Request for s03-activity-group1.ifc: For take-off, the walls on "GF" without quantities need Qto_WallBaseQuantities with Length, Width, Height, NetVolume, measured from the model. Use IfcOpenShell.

First a look at what the model holds.

```python
import ifcopenshell
import ifcopenshell.util.element
import ifcopenshell.util.unit

model = ifcopenshell.open("s03-activity-group1.ifc")
print(model.schema)
for unit_type in ("LENGTHUNIT", "AREAUNIT", "VOLUMEUNIT"):
    print(unit_type, ifcopenshell.util.unit.calculate_unit_scale(model, unit_type))
storey = next(s for s in model.by_type("IfcBuildingStorey") if s.Name == "GF")
walls = [e for e in ifcopenshell.util.element.get_decomposition(storey) if e.is_a("IfcWall")]
for e in sorted(walls, key=lambda e: e.id()):
    print(e.id(), e.is_a(), e.Name, list(ifcopenshell.util.element.get_psets(e, qtos_only=True)), sep=" | ")
```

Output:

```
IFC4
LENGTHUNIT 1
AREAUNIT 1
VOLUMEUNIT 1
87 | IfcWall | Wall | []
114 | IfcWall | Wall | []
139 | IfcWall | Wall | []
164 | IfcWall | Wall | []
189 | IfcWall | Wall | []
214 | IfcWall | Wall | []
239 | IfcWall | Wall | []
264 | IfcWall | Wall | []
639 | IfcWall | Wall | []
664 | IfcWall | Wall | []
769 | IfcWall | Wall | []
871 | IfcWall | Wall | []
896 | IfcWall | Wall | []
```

```python
import ifcopenshell
import ifcopenshell.api.pset
import ifcopenshell.geom
import ifcopenshell.util.element
import ifcopenshell.util.shape
import ifcopenshell.util.unit

model = ifcopenshell.open("s03-activity-group1.ifc")
unit_scale = ifcopenshell.util.unit.calculate_unit_scale(model)
volume_scale = ifcopenshell.util.unit.calculate_unit_scale(model, "VOLUMEUNIT")
settings = ifcopenshell.geom.settings()

storey = next(s for s in model.by_type("IfcBuildingStorey") if s.Name == "GF")
walls = [e for e in ifcopenshell.util.element.get_decomposition(storey) if e.is_a("IfcWall")]

for e in sorted(walls, key=lambda e: e.id()):
    if ifcopenshell.util.element.get_psets(e, qtos_only=True, should_inherit=False):
        continue
    # Geometry comes back in metres, in the element's own axes.
    shape = ifcopenshell.geom.create_shape(settings, e)
    values = {
        "Length": ifcopenshell.util.shape.get_x(shape.geometry) / unit_scale,
        "Width": ifcopenshell.util.shape.get_y(shape.geometry) / unit_scale,
        "Height": ifcopenshell.util.shape.get_z(shape.geometry) / unit_scale,
        "NetVolume": ifcopenshell.util.shape.get_volume(shape.geometry) / volume_scale,
    }
    qto = ifcopenshell.api.pset.add_qto(model, product=e, name="Qto_WallBaseQuantities")
    ifcopenshell.api.pset.edit_qto(model, qto=qto, properties=values)
    print(e.id(), {k: round(v, 3) for k, v in values.items()})

model.write("s03-activity-group1_rev.ifc")
```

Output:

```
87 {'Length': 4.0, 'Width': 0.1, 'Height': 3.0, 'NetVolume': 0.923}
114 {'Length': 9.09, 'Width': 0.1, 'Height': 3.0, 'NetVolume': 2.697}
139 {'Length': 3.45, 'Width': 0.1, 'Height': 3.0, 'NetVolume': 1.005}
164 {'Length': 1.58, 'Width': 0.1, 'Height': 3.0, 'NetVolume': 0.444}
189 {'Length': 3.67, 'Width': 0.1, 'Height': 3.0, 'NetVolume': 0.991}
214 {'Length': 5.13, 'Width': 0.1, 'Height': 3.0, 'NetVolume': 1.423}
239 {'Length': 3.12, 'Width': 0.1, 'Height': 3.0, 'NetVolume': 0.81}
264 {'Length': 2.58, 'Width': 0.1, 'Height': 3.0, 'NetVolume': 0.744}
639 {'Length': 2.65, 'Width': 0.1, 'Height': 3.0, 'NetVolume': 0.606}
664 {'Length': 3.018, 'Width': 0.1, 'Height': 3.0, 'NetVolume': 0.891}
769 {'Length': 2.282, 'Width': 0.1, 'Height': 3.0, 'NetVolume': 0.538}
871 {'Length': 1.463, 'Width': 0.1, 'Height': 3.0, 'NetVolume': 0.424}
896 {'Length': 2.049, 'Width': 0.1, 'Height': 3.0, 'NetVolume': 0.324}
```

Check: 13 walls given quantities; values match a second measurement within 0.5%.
